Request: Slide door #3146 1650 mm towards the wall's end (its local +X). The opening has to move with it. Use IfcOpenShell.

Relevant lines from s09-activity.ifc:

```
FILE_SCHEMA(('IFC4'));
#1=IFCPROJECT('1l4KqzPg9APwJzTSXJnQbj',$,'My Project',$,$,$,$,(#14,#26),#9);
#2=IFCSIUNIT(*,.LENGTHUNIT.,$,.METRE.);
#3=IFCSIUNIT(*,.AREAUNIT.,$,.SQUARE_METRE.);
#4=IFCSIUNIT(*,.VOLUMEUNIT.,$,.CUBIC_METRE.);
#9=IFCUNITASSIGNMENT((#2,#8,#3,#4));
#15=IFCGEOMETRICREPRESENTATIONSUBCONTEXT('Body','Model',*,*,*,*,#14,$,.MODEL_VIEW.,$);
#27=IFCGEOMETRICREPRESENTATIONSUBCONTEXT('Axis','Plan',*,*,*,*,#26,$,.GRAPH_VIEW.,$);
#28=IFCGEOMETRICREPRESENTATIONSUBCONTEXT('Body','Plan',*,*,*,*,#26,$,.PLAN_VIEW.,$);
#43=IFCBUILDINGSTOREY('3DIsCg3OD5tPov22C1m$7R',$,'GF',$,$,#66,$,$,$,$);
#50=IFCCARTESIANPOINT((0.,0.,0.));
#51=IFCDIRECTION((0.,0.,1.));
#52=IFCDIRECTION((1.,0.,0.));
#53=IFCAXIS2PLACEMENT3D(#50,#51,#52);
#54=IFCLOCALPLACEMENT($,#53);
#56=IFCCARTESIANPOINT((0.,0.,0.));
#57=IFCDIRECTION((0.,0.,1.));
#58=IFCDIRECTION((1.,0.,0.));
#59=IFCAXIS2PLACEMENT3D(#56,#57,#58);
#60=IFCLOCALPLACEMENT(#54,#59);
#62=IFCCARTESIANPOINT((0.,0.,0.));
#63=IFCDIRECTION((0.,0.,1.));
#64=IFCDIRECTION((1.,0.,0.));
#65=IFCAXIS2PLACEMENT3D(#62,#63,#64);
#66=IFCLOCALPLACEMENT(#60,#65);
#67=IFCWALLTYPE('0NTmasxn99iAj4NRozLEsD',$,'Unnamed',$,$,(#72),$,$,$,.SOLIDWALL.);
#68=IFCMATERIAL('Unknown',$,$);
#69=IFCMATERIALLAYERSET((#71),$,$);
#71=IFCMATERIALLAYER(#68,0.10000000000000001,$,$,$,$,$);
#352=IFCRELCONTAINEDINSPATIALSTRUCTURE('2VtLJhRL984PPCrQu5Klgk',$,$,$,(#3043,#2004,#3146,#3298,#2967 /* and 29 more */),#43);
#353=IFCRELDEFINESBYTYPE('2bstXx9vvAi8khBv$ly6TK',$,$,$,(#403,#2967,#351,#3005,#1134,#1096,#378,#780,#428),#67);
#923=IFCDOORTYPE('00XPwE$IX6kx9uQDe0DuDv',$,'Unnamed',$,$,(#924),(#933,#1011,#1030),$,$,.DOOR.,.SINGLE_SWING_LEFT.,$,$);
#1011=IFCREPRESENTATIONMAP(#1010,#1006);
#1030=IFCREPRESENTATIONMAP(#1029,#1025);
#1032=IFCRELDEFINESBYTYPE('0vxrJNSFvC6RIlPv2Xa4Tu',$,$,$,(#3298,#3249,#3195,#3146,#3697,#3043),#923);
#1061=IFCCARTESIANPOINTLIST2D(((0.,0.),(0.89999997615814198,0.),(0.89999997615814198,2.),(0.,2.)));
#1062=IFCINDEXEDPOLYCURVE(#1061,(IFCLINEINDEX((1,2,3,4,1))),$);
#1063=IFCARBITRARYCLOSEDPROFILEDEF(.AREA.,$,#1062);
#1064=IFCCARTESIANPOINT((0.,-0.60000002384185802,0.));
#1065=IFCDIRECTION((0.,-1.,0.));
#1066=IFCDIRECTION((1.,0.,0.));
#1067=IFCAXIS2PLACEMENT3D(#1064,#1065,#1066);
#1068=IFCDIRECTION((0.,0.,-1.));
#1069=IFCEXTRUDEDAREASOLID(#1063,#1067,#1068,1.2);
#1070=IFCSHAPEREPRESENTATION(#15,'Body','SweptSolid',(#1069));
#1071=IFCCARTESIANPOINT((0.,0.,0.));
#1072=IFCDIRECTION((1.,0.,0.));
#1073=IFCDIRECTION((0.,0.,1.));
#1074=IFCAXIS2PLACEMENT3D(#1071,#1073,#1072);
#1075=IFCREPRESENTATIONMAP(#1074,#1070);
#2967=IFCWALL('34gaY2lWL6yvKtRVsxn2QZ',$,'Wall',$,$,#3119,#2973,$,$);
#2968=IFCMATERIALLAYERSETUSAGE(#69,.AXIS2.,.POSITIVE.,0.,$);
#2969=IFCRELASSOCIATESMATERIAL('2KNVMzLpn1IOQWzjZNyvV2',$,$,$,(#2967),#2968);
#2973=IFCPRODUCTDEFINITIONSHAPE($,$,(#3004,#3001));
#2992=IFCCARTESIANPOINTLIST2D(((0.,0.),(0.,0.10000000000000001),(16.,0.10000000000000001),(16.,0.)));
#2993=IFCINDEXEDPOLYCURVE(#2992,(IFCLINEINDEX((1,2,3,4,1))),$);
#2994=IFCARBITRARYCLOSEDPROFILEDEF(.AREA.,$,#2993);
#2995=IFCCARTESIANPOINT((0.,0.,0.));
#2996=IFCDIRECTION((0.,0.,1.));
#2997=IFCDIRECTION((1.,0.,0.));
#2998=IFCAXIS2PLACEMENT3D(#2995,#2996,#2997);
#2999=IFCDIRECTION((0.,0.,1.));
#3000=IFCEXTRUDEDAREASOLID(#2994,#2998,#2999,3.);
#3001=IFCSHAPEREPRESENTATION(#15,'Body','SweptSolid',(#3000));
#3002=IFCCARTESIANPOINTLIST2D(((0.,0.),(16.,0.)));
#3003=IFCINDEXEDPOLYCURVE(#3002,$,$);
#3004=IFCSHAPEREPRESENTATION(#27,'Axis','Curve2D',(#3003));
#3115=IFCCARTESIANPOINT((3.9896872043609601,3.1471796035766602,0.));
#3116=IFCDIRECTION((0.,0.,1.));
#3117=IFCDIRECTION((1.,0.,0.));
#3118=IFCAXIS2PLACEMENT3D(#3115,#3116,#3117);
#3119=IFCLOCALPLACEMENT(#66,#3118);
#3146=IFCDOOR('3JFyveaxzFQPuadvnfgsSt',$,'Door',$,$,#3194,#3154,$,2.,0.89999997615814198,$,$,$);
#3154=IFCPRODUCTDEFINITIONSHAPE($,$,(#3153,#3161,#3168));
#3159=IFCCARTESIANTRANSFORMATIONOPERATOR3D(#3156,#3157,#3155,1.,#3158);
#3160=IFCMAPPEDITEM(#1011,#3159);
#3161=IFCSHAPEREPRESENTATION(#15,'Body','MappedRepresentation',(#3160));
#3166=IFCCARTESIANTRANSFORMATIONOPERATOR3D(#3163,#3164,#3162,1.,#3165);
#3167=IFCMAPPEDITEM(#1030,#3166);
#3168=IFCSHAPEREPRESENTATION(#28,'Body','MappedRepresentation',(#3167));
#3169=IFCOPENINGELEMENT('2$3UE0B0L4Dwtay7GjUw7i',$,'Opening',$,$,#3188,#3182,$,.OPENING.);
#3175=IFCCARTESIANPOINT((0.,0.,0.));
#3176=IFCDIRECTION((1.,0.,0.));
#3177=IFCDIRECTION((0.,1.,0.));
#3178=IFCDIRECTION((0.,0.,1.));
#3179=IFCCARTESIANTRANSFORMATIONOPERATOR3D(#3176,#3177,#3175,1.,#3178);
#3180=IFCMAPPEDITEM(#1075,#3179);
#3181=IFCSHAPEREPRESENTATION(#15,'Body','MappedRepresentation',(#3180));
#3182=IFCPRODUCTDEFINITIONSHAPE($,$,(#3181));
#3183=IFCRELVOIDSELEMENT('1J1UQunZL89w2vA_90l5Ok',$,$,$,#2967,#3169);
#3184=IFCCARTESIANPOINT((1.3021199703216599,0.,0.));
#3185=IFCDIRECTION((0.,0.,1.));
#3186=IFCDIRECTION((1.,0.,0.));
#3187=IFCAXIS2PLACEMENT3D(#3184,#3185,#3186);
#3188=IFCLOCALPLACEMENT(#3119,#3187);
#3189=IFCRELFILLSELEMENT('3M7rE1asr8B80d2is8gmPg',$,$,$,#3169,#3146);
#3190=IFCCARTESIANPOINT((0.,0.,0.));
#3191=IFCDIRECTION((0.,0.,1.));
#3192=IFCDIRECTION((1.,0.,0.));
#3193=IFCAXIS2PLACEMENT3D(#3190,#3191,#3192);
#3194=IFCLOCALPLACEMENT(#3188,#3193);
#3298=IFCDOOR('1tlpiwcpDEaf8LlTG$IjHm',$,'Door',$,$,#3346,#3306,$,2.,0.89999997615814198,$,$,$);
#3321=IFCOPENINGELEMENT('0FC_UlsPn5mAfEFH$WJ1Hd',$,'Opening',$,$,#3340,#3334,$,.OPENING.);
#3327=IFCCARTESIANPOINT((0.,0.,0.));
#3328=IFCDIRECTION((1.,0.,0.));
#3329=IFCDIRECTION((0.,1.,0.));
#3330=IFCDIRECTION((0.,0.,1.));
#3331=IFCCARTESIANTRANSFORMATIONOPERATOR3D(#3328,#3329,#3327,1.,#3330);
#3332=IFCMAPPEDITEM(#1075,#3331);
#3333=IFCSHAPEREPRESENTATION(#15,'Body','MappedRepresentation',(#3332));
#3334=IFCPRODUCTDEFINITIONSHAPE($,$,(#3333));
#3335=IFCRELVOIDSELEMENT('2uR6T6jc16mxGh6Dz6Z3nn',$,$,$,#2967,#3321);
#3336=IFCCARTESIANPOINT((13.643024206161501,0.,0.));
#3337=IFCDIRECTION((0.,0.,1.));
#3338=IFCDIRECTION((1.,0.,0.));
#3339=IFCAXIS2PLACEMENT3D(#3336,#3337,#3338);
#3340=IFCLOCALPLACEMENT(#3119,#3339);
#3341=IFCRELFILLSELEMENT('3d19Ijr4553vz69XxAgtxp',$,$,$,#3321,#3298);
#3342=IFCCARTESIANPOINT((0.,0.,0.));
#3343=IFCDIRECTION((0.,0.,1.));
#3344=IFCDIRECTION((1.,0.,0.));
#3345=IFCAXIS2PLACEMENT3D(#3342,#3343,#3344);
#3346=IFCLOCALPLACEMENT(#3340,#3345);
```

```python
import ifcopenshell
import ifcopenshell.api.geometry
import ifcopenshell.util.placement

model = ifcopenshell.open("s09-activity.ifc")

door = model.by_id(3146)
opening = door.FillsVoids[0].RelatingOpeningElement
wall = opening.VoidsElements[0].RelatingBuildingElement

wall_matrix = ifcopenshell.util.placement.get_local_placement(wall.ObjectPlacement)
shift = wall_matrix[:3, 0] * 1.65
before = ifcopenshell.util.placement.get_local_placement(door.ObjectPlacement)[:3, 3].copy()

# The door is placed relative to its opening, so it follows when the opening moves.
matrix = ifcopenshell.util.placement.get_local_placement(opening.ObjectPlacement)
matrix[:3, 3] += shift
ifcopenshell.api.geometry.edit_object_placement(
    model, product=opening, matrix=matrix, is_si=False, should_transform_children=True
)

after = ifcopenshell.util.placement.get_local_placement(door.ObjectPlacement)[:3, 3]
print("door moved by", (after - before).round(3) + 0.0)

model.write("s09-activity_rev.ifc")
```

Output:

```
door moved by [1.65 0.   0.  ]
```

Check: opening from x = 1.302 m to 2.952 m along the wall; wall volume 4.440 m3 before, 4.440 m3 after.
